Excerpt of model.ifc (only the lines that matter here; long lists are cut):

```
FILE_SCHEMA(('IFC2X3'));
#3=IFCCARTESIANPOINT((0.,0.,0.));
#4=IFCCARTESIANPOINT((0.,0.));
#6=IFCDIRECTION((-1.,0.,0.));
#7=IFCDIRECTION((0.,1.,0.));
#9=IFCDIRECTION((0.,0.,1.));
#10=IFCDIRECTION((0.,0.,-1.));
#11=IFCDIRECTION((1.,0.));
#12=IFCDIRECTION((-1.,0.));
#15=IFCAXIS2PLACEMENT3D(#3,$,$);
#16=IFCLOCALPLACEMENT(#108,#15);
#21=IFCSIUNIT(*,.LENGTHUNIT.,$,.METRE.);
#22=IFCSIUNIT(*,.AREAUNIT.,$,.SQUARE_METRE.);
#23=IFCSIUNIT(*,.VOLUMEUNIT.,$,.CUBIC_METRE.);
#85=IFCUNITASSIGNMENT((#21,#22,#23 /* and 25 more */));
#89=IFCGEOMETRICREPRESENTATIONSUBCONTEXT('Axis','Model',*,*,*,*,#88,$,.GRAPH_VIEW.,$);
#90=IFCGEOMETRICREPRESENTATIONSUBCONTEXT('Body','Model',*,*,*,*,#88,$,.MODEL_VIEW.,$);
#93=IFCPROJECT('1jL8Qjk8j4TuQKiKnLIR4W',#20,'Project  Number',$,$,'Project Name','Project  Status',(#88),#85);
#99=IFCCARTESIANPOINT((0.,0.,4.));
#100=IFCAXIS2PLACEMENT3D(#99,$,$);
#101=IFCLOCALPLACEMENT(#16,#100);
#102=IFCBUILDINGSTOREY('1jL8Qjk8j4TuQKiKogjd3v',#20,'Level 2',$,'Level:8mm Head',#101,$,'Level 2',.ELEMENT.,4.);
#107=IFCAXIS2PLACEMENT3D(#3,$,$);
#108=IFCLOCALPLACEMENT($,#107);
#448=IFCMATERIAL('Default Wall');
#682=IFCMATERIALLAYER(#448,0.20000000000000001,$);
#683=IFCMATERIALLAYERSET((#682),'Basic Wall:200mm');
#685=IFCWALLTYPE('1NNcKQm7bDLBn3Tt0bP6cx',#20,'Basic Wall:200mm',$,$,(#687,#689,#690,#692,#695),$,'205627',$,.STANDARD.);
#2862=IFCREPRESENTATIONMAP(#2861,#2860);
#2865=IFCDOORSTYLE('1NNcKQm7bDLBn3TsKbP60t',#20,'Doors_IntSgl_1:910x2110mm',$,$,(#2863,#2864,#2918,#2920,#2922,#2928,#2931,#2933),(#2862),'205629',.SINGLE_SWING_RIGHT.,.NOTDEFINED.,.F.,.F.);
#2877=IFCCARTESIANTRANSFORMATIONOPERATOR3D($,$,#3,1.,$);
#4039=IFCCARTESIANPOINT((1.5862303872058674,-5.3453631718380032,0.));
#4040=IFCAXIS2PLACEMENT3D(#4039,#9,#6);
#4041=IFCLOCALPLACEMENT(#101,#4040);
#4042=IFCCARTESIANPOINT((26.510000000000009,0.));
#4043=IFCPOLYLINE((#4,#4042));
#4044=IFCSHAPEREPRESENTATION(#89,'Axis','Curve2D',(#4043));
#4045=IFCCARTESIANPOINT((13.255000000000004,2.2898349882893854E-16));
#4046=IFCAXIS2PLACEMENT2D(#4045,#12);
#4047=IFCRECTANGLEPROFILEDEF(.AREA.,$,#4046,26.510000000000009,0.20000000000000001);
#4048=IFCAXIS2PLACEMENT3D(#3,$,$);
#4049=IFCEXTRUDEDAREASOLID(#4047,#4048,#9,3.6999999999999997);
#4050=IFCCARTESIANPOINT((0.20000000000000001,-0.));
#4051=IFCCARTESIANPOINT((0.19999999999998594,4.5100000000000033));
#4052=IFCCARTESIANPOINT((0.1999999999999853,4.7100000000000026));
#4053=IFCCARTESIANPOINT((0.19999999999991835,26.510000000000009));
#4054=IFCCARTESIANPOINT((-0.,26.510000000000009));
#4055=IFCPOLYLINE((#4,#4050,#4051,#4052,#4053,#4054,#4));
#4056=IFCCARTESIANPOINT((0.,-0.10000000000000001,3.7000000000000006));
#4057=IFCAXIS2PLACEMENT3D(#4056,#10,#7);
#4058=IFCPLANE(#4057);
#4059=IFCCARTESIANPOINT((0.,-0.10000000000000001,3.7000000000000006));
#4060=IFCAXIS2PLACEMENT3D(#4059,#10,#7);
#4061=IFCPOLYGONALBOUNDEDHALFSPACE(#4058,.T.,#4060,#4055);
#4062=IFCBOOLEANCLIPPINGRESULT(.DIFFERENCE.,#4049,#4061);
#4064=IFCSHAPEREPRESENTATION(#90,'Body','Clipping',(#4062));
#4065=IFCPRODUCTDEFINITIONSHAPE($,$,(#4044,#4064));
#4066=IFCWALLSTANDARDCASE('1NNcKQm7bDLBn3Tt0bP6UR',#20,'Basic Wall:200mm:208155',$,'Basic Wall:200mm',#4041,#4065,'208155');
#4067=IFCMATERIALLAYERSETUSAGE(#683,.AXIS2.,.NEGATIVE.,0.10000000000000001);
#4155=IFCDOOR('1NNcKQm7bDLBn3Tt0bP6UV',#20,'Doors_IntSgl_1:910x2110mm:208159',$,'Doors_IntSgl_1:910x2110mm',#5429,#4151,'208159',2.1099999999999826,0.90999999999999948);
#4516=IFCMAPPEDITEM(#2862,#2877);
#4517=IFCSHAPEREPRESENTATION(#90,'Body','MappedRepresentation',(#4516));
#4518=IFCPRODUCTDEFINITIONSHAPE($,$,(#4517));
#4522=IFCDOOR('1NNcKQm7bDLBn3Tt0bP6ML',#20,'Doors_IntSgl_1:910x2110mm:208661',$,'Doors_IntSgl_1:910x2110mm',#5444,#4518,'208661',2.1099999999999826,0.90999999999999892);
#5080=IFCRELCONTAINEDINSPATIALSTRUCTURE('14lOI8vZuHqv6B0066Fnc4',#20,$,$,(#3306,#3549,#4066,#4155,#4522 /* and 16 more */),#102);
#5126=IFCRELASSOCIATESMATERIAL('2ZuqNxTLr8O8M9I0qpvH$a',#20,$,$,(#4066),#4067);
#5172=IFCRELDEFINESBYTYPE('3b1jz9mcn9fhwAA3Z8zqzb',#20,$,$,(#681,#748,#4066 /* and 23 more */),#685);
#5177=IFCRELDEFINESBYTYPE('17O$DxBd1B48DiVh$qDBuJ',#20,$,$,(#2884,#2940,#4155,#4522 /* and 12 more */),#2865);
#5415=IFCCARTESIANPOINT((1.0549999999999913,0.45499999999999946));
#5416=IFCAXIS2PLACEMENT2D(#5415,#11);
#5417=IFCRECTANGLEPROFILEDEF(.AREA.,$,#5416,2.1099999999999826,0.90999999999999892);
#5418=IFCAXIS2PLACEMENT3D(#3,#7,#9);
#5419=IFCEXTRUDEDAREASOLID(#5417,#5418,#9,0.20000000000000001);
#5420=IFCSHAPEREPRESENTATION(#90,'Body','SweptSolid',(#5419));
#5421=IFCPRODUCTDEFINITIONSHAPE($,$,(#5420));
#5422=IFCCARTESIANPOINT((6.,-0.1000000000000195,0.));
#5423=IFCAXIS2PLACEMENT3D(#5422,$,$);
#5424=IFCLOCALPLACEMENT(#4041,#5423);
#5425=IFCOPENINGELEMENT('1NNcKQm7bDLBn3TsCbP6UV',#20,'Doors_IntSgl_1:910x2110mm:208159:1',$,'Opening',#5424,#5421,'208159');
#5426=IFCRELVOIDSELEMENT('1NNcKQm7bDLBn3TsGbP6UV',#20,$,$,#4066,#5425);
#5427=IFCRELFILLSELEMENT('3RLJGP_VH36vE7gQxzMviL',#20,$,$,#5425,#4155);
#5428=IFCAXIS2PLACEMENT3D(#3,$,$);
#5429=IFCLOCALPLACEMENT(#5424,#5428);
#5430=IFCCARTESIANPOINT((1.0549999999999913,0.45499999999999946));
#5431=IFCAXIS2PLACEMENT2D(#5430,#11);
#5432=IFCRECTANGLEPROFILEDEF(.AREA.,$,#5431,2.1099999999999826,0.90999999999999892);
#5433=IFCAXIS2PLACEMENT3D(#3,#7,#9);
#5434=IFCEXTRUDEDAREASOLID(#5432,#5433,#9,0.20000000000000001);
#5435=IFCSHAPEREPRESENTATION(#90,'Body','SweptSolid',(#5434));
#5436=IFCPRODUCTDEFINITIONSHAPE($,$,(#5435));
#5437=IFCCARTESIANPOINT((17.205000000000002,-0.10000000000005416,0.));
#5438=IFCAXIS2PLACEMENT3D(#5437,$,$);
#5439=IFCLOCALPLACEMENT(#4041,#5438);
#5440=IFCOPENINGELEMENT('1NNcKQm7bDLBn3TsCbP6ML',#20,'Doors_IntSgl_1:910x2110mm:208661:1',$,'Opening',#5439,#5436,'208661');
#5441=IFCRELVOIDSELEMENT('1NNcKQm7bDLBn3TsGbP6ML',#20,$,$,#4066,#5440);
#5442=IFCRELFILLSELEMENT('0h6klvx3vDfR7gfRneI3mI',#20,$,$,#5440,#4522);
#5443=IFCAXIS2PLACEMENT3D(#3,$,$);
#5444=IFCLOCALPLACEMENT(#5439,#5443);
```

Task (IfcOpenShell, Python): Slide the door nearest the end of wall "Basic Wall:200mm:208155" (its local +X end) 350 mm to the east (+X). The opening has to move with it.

```python
import ifcopenshell
import ifcopenshell.api.geometry
import ifcopenshell.util.placement
import ifcopenshell.util.unit

model = ifcopenshell.open("model.ifc")
unit_scale = ifcopenshell.util.unit.calculate_unit_scale(model)

door = model.by_id(4522)
opening = door.FillsVoids[0].RelatingOpeningElement
wall = opening.VoidsElements[0].RelatingBuildingElement

wall_matrix = ifcopenshell.util.placement.get_local_placement(wall.ObjectPlacement)
shift = wall_matrix[:3, 0] * -0.35 / unit_scale
before = ifcopenshell.util.placement.get_local_placement(door.ObjectPlacement)[:3, 3].copy()

# The door is placed relative to its opening, so it follows when the opening moves.
matrix = ifcopenshell.util.placement.get_local_placement(opening.ObjectPlacement)
matrix[:3, 3] += shift
ifcopenshell.api.geometry.edit_object_placement(
    model, product=opening, matrix=matrix, is_si=False, should_transform_children=True
)

after = ifcopenshell.util.placement.get_local_placement(door.ObjectPlacement)[:3, 3]
print("door moved by", (after - before).round(3) + 0.0)

model.write("model_edited.ifc")
```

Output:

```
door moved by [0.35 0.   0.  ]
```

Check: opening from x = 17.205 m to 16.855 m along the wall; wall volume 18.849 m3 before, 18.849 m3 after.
